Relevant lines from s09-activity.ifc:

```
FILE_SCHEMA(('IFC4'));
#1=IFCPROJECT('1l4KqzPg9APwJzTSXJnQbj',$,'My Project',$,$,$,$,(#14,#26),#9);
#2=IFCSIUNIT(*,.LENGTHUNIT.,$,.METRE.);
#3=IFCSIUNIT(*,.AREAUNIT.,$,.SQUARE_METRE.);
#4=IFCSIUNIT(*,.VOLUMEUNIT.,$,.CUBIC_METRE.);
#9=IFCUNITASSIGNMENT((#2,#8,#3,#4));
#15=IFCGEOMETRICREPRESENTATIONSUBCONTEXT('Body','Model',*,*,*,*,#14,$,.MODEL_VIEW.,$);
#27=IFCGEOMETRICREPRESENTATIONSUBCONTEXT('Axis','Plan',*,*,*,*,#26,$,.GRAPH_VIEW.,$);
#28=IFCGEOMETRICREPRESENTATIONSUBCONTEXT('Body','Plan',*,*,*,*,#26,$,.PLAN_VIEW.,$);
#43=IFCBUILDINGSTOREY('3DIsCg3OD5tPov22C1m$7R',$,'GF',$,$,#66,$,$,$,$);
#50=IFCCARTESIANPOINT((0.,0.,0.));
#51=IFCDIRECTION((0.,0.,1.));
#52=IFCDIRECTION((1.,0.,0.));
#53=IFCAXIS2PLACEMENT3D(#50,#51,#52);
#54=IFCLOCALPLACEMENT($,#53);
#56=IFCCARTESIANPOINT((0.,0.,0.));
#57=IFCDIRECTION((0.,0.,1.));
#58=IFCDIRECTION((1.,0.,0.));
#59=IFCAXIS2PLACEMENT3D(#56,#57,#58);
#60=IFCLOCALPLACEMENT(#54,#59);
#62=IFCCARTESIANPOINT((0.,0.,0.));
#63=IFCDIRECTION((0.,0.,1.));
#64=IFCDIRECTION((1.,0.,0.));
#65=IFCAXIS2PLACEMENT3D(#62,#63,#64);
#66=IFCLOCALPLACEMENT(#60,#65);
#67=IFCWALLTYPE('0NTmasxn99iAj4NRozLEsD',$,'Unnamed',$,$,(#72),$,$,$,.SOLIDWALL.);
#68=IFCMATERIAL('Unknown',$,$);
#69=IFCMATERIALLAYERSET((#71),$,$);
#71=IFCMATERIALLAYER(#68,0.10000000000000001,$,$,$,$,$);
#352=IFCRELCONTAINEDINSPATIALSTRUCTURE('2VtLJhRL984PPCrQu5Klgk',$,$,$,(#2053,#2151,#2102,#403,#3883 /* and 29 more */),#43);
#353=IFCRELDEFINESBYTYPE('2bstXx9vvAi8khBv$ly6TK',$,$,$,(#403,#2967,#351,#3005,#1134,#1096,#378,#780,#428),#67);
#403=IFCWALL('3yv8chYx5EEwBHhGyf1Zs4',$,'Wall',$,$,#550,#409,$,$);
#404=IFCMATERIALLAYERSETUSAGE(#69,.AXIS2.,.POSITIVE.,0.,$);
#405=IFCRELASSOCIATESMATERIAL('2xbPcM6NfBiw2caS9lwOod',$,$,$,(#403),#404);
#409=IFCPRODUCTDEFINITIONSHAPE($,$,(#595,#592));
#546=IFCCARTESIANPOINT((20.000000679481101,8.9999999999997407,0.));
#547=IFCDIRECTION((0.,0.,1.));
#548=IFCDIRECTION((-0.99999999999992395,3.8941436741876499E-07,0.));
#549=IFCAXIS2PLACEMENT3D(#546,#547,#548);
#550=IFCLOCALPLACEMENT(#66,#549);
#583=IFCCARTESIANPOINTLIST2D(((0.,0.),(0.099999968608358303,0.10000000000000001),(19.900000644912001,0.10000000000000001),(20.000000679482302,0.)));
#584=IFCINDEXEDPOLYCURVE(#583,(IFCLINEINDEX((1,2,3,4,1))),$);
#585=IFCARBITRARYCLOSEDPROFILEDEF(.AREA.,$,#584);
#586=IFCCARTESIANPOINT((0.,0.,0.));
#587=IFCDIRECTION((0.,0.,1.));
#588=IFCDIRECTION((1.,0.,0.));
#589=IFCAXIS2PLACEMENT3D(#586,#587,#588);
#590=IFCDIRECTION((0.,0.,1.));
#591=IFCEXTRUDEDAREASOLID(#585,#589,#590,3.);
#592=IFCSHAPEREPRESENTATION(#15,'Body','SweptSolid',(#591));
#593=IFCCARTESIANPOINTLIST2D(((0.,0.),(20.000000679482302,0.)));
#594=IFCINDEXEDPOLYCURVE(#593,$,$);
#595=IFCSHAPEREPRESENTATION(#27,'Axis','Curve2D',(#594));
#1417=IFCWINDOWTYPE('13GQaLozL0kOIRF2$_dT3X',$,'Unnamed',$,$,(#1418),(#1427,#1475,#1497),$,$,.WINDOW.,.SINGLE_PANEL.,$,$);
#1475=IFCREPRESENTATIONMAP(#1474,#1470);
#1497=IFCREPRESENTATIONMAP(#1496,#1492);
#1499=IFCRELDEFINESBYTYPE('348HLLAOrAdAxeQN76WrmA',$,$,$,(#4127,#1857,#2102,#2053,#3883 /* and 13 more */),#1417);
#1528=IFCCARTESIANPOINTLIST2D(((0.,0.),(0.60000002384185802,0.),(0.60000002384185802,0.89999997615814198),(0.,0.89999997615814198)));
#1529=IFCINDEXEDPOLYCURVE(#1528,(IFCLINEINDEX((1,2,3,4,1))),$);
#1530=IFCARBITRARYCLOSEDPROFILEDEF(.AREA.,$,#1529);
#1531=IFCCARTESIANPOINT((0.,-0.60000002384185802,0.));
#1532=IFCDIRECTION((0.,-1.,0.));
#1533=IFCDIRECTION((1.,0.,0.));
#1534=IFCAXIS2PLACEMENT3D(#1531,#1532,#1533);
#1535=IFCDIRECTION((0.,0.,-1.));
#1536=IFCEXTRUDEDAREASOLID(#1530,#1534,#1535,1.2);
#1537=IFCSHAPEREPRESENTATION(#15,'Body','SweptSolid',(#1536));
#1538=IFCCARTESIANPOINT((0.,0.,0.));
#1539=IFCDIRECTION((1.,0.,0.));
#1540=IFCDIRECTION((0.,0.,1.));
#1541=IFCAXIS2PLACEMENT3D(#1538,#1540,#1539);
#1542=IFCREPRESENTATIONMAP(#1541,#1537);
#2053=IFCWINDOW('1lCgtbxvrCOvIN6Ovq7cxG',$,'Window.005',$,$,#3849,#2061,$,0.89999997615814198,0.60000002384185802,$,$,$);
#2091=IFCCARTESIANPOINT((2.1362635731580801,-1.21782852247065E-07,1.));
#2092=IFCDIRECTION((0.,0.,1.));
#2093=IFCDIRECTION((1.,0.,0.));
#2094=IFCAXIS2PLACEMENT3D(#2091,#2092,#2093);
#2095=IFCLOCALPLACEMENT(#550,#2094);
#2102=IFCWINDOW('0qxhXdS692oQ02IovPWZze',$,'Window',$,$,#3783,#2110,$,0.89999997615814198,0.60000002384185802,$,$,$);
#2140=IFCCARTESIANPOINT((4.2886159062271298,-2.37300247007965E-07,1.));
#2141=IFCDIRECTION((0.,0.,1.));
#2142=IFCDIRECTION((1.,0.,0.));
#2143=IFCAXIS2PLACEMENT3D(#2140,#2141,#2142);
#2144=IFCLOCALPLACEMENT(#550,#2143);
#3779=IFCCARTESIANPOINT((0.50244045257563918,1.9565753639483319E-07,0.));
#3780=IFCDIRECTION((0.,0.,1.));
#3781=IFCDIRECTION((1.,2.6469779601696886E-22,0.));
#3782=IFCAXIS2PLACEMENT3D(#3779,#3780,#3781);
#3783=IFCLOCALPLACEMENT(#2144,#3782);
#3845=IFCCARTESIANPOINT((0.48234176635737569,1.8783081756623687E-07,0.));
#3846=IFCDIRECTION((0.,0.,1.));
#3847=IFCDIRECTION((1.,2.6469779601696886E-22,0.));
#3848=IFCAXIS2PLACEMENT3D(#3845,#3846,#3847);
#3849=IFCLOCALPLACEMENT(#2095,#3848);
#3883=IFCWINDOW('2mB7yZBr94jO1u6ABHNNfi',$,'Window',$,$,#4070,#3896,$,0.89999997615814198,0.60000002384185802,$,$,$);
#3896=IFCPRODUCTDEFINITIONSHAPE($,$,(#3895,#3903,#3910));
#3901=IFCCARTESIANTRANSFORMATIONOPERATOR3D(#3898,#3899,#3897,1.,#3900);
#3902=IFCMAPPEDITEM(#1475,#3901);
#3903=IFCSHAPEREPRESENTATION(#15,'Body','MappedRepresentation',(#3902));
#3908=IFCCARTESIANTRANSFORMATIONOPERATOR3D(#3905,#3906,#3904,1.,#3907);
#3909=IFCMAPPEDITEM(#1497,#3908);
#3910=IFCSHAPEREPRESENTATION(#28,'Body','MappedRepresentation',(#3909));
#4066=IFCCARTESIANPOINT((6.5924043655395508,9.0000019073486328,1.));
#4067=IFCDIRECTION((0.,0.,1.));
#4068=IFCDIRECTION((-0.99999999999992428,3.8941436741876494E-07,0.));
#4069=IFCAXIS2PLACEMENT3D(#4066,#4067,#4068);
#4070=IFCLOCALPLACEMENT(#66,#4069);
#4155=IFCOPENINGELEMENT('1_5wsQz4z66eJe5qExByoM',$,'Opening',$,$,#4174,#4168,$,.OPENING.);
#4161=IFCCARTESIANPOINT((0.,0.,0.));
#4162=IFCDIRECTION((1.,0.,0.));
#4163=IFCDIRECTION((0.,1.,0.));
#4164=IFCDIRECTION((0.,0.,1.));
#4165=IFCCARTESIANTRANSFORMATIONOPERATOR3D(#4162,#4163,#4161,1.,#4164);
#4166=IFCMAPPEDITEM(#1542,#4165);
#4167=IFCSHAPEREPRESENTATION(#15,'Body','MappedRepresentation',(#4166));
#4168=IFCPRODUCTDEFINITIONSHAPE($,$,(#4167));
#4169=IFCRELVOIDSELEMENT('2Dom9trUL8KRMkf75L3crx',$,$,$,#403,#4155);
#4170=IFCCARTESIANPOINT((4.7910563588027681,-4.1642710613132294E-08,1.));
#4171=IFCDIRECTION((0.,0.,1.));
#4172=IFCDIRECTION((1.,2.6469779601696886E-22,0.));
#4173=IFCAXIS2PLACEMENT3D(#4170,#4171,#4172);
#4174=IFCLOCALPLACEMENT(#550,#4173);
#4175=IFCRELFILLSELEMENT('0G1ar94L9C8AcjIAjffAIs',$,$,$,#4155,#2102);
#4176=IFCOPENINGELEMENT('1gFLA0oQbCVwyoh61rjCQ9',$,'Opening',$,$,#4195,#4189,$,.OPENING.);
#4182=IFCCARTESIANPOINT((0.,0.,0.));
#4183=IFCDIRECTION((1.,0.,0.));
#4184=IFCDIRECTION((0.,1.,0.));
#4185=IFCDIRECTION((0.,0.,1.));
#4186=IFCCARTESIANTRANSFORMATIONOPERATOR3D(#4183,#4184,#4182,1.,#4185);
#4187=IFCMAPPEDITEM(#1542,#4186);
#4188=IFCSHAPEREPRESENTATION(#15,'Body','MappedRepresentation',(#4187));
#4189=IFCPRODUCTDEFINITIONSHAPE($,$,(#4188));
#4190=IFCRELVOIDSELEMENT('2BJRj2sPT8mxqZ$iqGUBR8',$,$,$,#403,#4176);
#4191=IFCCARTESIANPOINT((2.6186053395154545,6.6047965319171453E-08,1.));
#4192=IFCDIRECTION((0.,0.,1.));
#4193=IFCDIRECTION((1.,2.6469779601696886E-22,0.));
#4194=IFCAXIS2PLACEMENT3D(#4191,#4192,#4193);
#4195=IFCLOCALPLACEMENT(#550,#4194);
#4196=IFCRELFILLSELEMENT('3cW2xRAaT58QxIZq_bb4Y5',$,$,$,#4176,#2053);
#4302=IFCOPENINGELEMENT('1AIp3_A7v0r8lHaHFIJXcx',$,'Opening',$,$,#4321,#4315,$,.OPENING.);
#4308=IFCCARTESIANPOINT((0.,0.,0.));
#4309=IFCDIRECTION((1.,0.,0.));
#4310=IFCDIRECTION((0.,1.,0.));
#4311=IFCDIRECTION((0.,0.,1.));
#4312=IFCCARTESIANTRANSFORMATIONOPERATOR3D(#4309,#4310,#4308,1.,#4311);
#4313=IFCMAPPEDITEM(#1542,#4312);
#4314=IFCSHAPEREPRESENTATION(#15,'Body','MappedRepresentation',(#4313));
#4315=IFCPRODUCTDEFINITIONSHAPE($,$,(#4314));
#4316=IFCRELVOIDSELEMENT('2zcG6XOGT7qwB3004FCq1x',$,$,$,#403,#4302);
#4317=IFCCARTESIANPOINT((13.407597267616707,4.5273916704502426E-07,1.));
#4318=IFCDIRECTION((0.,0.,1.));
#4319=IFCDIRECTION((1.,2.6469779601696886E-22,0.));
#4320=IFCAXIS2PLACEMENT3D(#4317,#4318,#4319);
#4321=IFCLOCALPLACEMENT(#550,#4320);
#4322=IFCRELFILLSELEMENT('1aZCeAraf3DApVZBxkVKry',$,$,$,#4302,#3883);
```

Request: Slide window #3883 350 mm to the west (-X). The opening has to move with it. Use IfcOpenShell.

```python
import ifcopenshell
import ifcopenshell.api.geometry
import ifcopenshell.util.placement
import ifcopenshell.util.unit

model = ifcopenshell.open("s09-activity.ifc")
unit_scale = ifcopenshell.util.unit.calculate_unit_scale(model)

window = model.by_guid("2mB7yZBr94jO1u6ABHNNfi")
opening = window.FillsVoids[0].RelatingOpeningElement
wall = opening.VoidsElements[0].RelatingBuildingElement

wall_matrix = ifcopenshell.util.placement.get_local_placement(wall.ObjectPlacement)
shift = wall_matrix[:3, 0] * 0.35 / unit_scale
before = ifcopenshell.util.placement.get_local_placement(window.ObjectPlacement)[:3, 3].copy()

# The window is not placed relative to its opening, so move both.
for product in (opening, window):
    matrix = ifcopenshell.util.placement.get_local_placement(product.ObjectPlacement)
    matrix[:3, 3] += shift
    ifcopenshell.api.geometry.edit_object_placement(model, product=product, matrix=matrix, is_si=False)

after = ifcopenshell.util.placement.get_local_placement(window.ObjectPlacement)[:3, 3]
print("window moved by", (after - before).round(3) + 0.0)

model.write("s09-activity_rev.ifc")
```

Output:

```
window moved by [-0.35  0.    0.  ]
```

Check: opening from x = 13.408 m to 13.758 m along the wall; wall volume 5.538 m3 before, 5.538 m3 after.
